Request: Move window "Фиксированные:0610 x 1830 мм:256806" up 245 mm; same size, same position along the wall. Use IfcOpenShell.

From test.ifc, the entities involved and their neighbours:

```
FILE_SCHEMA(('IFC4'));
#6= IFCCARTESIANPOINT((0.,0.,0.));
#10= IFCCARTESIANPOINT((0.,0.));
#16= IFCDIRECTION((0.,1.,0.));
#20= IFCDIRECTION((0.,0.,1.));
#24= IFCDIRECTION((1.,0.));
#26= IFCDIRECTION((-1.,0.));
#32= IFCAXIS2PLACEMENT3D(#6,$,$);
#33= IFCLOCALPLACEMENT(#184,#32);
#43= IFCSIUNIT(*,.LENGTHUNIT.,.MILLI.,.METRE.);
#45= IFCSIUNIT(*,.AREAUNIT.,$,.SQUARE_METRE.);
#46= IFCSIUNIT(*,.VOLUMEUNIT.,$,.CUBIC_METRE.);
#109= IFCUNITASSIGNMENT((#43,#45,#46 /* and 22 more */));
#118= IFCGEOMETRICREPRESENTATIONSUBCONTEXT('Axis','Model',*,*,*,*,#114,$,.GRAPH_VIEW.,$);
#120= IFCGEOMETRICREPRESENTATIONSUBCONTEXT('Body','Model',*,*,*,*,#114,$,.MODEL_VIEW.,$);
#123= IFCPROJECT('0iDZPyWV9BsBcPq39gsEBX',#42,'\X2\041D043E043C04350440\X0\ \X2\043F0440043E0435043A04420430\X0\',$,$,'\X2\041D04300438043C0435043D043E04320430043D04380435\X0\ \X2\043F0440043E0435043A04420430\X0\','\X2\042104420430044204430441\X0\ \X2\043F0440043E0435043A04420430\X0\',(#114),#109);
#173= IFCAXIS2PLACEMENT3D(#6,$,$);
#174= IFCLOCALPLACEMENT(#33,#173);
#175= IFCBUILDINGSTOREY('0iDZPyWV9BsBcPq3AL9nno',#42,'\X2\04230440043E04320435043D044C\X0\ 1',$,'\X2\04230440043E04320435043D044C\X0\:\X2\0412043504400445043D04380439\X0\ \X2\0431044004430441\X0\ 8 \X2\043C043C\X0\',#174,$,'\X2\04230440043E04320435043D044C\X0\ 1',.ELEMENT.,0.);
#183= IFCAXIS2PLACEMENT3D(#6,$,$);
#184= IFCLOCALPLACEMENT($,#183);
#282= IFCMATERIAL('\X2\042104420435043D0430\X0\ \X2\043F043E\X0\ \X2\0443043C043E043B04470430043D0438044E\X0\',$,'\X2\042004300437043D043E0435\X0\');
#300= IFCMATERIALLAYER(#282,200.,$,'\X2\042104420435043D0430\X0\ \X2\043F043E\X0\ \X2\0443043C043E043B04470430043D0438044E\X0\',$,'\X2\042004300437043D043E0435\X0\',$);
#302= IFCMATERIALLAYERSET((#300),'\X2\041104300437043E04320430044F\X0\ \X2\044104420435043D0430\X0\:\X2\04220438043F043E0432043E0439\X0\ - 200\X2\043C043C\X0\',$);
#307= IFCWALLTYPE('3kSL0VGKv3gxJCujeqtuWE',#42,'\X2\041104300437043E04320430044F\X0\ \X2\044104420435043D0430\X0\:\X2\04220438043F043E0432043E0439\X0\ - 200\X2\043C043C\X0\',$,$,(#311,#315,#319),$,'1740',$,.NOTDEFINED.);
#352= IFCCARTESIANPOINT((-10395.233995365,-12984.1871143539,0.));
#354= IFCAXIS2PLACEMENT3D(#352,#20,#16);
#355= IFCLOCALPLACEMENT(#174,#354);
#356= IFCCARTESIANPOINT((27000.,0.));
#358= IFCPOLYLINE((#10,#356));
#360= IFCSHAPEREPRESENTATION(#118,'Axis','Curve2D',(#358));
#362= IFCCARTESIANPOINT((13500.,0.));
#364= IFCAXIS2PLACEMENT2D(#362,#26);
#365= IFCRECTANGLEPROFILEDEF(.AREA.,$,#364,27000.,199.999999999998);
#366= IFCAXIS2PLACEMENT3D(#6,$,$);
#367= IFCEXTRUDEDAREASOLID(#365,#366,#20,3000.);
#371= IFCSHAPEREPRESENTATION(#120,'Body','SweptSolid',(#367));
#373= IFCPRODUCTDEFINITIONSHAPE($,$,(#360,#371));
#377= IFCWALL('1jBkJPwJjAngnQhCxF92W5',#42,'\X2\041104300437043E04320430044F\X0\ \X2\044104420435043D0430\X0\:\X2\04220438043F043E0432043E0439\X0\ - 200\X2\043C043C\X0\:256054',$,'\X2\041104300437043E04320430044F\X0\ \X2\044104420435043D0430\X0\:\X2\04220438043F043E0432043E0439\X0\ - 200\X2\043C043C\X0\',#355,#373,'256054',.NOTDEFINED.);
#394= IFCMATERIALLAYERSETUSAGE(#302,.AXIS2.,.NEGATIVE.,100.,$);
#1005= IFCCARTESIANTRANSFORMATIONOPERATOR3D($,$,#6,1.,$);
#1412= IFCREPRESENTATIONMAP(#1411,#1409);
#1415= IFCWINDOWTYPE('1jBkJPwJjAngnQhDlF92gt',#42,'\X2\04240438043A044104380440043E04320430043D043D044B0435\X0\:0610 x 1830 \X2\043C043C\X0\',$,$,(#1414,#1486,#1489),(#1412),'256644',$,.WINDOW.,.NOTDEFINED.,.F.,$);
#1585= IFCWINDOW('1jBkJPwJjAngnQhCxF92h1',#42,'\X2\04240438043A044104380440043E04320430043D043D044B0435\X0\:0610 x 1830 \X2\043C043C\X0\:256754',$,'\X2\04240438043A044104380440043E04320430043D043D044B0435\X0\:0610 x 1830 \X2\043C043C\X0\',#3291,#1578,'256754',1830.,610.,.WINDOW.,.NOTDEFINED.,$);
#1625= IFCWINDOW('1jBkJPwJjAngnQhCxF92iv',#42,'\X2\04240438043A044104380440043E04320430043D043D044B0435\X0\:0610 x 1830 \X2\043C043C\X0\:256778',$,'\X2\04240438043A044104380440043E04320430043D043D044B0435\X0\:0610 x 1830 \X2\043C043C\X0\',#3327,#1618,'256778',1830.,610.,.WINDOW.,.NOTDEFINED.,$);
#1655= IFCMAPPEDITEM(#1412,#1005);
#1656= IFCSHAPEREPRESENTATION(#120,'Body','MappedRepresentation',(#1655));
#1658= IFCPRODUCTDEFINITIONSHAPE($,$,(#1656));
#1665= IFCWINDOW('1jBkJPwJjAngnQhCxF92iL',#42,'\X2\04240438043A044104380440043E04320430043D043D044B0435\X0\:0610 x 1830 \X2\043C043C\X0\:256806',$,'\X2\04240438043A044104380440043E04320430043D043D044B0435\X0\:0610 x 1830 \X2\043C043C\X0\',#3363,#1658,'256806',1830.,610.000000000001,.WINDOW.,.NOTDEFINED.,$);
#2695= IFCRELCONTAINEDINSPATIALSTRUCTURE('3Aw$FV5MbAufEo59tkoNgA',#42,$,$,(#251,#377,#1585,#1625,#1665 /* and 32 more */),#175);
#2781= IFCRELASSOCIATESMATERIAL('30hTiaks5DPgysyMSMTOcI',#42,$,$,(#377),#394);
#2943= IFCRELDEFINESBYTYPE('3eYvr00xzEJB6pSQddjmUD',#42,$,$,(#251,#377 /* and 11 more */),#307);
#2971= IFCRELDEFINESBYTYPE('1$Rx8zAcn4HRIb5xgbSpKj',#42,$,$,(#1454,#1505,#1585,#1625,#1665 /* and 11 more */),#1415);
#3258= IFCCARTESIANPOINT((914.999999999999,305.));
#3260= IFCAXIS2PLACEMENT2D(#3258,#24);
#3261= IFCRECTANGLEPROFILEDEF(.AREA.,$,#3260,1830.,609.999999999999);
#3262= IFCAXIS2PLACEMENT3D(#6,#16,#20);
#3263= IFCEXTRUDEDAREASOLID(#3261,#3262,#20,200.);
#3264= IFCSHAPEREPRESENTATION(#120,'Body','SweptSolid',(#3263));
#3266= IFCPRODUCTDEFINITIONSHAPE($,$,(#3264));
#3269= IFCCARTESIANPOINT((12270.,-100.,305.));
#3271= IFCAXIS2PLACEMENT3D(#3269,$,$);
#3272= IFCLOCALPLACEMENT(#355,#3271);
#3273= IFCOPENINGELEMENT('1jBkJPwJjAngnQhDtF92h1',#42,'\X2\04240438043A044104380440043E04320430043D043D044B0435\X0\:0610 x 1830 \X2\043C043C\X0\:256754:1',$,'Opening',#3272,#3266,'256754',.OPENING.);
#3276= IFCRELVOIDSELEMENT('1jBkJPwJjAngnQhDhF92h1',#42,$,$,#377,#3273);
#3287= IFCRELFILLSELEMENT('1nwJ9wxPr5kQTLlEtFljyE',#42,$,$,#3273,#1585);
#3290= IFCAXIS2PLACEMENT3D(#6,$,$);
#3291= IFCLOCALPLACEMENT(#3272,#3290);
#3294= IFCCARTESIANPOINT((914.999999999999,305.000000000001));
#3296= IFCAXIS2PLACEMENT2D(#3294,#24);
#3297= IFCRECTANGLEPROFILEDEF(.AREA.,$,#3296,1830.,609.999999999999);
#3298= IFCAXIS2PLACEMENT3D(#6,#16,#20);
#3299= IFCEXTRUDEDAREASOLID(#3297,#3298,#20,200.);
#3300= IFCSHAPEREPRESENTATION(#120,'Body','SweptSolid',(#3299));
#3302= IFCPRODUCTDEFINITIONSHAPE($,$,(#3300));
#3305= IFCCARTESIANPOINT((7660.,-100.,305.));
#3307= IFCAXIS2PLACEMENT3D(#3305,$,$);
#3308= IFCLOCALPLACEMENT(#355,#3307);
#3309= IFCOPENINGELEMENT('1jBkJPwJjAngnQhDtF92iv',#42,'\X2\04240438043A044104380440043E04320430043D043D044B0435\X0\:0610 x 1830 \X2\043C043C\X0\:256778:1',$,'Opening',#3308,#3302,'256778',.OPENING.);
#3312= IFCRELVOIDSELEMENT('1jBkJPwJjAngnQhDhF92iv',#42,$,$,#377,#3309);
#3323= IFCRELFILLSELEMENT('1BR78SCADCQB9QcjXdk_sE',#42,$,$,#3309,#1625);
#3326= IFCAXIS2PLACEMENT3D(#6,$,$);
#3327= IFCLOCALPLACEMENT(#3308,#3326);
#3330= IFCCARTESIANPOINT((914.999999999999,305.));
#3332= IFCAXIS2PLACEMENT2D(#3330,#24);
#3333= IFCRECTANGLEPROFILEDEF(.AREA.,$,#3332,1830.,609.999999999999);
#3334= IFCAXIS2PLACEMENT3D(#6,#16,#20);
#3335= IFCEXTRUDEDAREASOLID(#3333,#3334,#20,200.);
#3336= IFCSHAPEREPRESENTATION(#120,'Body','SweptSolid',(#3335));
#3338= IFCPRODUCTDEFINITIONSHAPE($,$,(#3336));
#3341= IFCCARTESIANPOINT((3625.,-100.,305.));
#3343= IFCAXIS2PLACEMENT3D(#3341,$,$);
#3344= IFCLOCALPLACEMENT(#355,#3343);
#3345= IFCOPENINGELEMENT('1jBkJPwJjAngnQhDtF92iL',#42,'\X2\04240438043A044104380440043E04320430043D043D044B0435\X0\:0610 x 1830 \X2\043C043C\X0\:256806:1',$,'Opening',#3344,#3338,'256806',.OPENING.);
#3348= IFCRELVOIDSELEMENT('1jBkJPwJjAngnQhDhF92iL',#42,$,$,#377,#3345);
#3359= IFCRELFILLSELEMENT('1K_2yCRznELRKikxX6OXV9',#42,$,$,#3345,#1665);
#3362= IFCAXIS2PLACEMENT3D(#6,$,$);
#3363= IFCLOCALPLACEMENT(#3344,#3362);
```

```python
import numpy as np
import ifcopenshell
import ifcopenshell.api.geometry
import ifcopenshell.util.placement
import ifcopenshell.util.unit

model = ifcopenshell.open("test.ifc")
unit_scale = ifcopenshell.util.unit.calculate_unit_scale(model)

window = model.by_guid("1jBkJPwJjAngnQhCxF92iL")
opening = window.FillsVoids[0].RelatingOpeningElement
dz = 245.0

shift = np.array([0.0, 0.0, dz])
# The window is placed relative to its opening, so it follows when the opening moves.
matrix = ifcopenshell.util.placement.get_local_placement(opening.ObjectPlacement)
matrix[:3, 3] += shift
ifcopenshell.api.geometry.edit_object_placement(
    model, product=opening, matrix=matrix, is_si=False, should_transform_children=True
)

print(f"moved by {dz * unit_scale:+.3f} m")

model.write("test_rev.ifc")
```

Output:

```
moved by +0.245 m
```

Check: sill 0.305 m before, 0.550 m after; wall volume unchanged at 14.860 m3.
